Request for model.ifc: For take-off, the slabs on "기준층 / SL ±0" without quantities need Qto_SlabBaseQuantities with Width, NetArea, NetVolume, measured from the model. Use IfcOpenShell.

First a look at what the model holds.

```python
import ifcopenshell
import ifcopenshell.util.element
import ifcopenshell.util.unit

model = ifcopenshell.open("model.ifc")
print(model.schema)
for unit_type in ("LENGTHUNIT", "AREAUNIT", "VOLUMEUNIT"):
    print(unit_type, ifcopenshell.util.unit.calculate_unit_scale(model, unit_type))
storey = next(s for s in model.by_type("IfcBuildingStorey") if s.Name == "기준층 / SL ±0")
slabs = [e for e in ifcopenshell.util.element.get_decomposition(storey) if e.is_a("IfcSlab")]
for e in sorted(slabs, key=lambda e: e.id()):
    print(e.id(), e.is_a(), e.Name, list(ifcopenshell.util.element.get_psets(e, qtos_only=True)), sep=" | ")
```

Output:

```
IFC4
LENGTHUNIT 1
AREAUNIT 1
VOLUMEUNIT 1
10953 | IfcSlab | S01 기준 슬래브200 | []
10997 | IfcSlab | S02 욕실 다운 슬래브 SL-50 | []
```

```python
import ifcopenshell
import ifcopenshell.api.pset
import ifcopenshell.geom
import ifcopenshell.util.element
import ifcopenshell.util.shape
import ifcopenshell.util.unit

model = ifcopenshell.open("model.ifc")
unit_scale = ifcopenshell.util.unit.calculate_unit_scale(model)
area_scale = ifcopenshell.util.unit.calculate_unit_scale(model, "AREAUNIT")
volume_scale = ifcopenshell.util.unit.calculate_unit_scale(model, "VOLUMEUNIT")
settings = ifcopenshell.geom.settings()

storey = next(s for s in model.by_type("IfcBuildingStorey") if s.Name == "기준층 / SL ±0")
slabs = [e for e in ifcopenshell.util.element.get_decomposition(storey) if e.is_a("IfcSlab")]

for e in sorted(slabs, key=lambda e: e.id()):
    if ifcopenshell.util.element.get_psets(e, qtos_only=True, should_inherit=False):
        continue
    # Geometry comes back in metres, in the element's own axes.
    shape = ifcopenshell.geom.create_shape(settings, e)
    values = {
        "Width": ifcopenshell.util.shape.get_z(shape.geometry) / unit_scale,
        "NetArea": ifcopenshell.util.shape.get_footprint_area(shape.geometry) / area_scale,
        "NetVolume": ifcopenshell.util.shape.get_volume(shape.geometry) / volume_scale,
    }
    qto = ifcopenshell.api.pset.add_qto(model, product=e, name="Qto_SlabBaseQuantities")
    ifcopenshell.api.pset.edit_qto(model, qto=qto, properties=values)
    print(e.id(), {k: round(v, 3) for k, v in values.items()})

model.write("model_v2.ifc")
```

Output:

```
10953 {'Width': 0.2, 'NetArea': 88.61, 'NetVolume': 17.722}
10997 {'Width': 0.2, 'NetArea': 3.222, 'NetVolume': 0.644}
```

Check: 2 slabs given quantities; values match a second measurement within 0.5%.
